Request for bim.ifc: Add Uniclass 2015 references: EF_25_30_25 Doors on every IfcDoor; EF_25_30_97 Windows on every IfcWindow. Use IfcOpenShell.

First a look at what the model holds.

```python
import ifcopenshell

model = ifcopenshell.open("bim.ifc")
print(model.schema)
print("classifications:", [c.Name for c in model.by_type("IfcClassification")])
for ifc_class in ("IfcDoor", "IfcRoof", "IfcStair", "IfcWall", "IfcWindow"):
    print(ifc_class, len(model.by_type(ifc_class)))
```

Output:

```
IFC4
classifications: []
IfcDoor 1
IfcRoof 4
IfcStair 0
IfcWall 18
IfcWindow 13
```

```python
import ifcopenshell
import ifcopenshell.api.classification

model = ifcopenshell.open("bim.ifc")

system = ifcopenshell.api.classification.add_classification(model, classification="Uniclass 2015")

codes = {
    "IfcDoor": ("EF_25_30_25", "Doors"),
    "IfcWindow": ("EF_25_30_97", "Windows"),
}
for ifc_class, (code, name) in codes.items():
    products = model.by_type(ifc_class)
    ifcopenshell.api.classification.add_reference(
        model, products=products, classification=system, identification=code, name=name
    )
    print(code, len(products))

model.write("bim_updated.ifc")
```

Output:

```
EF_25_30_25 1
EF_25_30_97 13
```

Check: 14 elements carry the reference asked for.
